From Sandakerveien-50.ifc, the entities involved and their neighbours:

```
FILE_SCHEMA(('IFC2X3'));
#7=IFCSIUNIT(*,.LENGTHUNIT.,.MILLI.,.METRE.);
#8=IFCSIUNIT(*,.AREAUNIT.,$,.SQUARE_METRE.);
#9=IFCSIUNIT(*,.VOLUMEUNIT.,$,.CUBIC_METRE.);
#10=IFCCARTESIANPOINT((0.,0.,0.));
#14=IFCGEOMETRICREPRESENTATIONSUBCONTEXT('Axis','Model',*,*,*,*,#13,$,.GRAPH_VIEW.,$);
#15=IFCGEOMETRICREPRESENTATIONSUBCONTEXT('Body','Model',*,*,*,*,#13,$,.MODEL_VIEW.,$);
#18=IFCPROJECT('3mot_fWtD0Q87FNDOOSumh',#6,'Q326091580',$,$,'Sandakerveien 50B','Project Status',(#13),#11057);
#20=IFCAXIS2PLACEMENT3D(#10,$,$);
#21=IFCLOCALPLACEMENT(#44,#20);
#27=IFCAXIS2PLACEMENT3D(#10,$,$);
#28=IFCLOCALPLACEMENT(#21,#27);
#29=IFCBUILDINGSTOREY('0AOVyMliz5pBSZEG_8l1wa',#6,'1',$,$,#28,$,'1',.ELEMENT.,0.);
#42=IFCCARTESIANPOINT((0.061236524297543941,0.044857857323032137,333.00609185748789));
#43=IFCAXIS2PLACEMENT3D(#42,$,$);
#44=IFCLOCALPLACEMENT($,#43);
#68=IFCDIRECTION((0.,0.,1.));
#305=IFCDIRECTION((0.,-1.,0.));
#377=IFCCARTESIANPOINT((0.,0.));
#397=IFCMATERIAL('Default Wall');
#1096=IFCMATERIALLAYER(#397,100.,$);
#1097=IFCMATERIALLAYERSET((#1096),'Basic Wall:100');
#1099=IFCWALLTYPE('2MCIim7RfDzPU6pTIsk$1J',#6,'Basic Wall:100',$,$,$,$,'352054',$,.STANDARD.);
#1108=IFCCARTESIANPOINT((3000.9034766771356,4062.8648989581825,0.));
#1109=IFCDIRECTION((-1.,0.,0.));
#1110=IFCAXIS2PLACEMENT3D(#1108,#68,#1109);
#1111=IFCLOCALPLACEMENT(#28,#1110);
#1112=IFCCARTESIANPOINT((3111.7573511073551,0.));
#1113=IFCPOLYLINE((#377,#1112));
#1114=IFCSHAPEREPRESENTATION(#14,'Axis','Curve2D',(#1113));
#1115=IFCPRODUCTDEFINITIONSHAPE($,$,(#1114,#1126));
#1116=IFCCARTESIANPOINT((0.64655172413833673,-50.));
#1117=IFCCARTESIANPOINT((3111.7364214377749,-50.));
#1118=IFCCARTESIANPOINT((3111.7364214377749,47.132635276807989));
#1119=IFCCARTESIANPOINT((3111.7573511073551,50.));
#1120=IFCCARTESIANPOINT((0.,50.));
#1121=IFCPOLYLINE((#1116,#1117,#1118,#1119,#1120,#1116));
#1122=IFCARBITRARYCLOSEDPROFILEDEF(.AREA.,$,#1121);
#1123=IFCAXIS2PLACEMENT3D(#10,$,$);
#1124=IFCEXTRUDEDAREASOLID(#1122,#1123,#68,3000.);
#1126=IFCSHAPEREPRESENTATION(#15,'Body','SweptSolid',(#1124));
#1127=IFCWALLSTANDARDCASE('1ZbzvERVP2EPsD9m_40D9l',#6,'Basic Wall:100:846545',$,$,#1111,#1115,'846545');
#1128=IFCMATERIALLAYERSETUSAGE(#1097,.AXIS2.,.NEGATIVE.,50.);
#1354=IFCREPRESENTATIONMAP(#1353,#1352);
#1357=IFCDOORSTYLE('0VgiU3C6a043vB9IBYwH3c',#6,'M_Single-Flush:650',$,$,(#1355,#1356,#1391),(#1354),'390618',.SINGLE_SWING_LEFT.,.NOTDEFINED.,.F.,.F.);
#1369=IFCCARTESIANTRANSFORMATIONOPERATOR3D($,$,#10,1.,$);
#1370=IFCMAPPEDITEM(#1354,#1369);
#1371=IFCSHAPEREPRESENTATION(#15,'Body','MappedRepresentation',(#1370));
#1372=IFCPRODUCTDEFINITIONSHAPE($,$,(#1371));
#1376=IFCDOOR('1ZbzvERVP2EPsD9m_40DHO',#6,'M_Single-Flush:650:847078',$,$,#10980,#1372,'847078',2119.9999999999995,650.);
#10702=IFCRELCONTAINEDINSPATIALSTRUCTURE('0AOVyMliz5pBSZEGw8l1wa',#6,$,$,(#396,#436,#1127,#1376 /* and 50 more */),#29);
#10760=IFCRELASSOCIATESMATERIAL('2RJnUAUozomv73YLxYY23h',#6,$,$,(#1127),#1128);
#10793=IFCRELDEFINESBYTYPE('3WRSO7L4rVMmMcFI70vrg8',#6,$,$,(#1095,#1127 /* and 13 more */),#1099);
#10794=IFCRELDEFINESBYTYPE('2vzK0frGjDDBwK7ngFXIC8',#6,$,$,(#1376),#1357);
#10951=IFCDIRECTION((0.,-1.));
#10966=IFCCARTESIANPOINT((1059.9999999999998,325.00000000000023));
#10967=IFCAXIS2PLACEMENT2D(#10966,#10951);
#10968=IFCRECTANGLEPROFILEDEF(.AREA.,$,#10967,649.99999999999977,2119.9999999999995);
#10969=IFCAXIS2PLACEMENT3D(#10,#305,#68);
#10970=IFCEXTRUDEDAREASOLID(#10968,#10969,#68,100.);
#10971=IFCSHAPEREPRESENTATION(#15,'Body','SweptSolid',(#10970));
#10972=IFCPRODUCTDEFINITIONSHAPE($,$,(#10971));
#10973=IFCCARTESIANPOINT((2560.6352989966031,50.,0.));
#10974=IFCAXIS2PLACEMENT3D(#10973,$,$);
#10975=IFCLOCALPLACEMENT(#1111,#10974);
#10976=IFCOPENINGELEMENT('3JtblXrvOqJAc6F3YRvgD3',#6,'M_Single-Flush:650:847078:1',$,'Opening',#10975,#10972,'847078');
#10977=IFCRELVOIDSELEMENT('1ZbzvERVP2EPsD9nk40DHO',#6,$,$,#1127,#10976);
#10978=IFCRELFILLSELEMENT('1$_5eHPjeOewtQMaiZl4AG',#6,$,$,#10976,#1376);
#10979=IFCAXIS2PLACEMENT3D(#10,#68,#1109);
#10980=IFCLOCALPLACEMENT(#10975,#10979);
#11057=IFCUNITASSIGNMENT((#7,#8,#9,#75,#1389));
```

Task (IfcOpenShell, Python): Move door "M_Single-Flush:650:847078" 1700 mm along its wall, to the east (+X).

```python
import ifcopenshell
import ifcopenshell.api.geometry
import ifcopenshell.util.placement

model = ifcopenshell.open("Sandakerveien-50.ifc")

door = model.by_guid("1ZbzvERVP2EPsD9m_40DHO")
opening = door.FillsVoids[0].RelatingOpeningElement
wall = opening.VoidsElements[0].RelatingBuildingElement

wall_matrix = ifcopenshell.util.placement.get_local_placement(wall.ObjectPlacement)
shift = wall_matrix[:3, 0] * -1700.0
before = ifcopenshell.util.placement.get_local_placement(door.ObjectPlacement)[:3, 3].copy()

# The door is placed relative to its opening, so it follows when the opening moves.
matrix = ifcopenshell.util.placement.get_local_placement(opening.ObjectPlacement)
matrix[:3, 3] += shift
ifcopenshell.api.geometry.edit_object_placement(
    model, product=opening, matrix=matrix, is_si=False, should_transform_children=True
)

after = ifcopenshell.util.placement.get_local_placement(door.ObjectPlacement)[:3, 3]
print("door moved by", (after - before).round(3) + 0.0)

model.write("Sandakerveien-50_rev.ifc")
```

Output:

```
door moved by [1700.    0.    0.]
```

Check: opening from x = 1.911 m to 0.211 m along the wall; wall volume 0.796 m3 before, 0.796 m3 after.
